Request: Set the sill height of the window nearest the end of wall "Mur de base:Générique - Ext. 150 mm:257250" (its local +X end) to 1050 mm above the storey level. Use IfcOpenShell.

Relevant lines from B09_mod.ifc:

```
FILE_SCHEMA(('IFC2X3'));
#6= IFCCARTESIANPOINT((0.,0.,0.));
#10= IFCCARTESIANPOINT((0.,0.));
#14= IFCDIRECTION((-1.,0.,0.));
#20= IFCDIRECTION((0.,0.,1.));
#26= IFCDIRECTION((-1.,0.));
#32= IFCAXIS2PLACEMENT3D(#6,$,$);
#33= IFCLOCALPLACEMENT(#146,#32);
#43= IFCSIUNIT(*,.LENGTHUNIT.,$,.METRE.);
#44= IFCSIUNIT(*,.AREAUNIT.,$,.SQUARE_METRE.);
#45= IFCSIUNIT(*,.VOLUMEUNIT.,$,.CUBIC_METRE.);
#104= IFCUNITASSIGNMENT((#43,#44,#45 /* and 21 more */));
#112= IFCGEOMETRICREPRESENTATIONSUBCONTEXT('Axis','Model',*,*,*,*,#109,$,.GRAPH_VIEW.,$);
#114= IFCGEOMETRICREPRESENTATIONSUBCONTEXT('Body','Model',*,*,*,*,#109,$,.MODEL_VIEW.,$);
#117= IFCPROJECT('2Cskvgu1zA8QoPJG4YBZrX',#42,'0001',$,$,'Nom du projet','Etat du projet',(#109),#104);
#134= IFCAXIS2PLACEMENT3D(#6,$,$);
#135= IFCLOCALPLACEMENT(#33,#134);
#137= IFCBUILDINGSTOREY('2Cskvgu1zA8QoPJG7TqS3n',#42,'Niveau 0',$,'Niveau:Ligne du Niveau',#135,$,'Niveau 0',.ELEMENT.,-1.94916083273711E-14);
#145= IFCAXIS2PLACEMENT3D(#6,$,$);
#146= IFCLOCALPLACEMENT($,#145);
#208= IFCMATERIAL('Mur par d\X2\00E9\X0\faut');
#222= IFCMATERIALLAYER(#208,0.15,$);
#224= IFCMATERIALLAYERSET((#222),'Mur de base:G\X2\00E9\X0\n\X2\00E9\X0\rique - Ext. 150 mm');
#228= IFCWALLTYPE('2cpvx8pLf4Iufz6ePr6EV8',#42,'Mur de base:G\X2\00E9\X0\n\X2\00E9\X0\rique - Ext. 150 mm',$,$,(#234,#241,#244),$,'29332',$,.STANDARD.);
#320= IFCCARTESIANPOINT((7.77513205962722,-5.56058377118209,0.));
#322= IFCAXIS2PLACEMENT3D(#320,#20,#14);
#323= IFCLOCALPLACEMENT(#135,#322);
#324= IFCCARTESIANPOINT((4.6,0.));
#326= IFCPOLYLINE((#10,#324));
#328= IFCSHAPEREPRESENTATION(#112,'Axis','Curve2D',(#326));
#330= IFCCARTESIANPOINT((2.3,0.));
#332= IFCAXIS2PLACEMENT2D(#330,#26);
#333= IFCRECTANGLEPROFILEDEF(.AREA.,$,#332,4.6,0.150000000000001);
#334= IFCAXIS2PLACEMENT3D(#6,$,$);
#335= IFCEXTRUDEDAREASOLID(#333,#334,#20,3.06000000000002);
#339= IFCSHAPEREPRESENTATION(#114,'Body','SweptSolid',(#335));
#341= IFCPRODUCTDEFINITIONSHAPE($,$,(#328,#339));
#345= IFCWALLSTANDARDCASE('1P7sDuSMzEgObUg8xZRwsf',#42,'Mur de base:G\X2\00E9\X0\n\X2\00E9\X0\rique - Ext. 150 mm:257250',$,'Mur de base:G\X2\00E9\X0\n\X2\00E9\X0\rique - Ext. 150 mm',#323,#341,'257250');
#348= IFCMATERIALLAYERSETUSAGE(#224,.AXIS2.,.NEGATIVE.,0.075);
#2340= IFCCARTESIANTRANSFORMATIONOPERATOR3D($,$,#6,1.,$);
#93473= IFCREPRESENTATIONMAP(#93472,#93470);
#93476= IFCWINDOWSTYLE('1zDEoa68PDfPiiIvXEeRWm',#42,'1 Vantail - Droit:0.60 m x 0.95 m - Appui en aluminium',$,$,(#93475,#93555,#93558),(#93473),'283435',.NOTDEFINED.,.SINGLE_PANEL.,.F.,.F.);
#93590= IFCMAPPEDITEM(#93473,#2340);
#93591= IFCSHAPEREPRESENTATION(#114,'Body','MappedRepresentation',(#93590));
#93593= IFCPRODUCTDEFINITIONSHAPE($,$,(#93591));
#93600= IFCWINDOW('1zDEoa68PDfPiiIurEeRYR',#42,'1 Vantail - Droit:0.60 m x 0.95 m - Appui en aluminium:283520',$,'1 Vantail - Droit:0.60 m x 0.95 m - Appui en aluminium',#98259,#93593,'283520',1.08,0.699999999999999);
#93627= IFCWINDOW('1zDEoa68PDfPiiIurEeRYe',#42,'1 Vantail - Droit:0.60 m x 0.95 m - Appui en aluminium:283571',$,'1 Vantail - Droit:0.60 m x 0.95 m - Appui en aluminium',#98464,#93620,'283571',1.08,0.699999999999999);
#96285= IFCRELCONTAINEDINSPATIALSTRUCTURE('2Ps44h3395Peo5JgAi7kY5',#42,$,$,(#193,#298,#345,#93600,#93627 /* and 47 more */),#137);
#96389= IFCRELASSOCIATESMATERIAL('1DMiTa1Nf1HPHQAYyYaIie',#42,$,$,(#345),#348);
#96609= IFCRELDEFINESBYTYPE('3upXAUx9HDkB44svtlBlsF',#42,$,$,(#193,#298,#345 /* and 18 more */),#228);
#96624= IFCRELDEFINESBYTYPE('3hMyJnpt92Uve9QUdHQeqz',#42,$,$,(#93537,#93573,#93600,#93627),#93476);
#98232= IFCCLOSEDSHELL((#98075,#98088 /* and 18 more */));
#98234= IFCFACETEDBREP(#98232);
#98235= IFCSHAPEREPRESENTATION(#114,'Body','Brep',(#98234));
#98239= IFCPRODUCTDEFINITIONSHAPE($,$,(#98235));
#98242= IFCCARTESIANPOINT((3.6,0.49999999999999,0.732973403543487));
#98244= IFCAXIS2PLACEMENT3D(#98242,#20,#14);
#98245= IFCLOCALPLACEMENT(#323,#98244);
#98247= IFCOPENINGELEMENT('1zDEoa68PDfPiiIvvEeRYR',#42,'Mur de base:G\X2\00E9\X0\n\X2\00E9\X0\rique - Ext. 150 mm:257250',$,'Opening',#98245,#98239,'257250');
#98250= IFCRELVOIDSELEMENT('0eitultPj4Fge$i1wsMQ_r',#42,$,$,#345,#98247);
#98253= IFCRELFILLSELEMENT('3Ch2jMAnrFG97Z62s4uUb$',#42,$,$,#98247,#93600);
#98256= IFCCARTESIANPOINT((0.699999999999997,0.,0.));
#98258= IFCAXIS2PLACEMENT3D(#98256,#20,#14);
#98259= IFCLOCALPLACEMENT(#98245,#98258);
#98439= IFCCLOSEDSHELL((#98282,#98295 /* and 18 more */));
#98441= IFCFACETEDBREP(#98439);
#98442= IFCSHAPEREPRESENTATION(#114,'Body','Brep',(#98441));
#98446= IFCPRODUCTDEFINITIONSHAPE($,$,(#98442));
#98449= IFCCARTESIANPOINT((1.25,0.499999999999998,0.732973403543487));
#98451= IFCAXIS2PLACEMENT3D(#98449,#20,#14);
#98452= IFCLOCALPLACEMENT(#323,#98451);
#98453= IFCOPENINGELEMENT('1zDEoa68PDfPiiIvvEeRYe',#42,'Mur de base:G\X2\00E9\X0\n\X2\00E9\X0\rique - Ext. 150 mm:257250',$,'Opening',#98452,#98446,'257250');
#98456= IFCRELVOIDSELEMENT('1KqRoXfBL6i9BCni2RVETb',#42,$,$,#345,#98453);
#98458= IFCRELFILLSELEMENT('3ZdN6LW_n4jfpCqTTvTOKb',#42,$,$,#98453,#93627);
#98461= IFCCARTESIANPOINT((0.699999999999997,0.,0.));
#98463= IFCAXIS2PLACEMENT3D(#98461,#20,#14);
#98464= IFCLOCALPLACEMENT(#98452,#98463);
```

```python
import numpy as np
import ifcopenshell
import ifcopenshell.api.geometry
import ifcopenshell.geom
import ifcopenshell.util.element
import ifcopenshell.util.placement
import ifcopenshell.util.shape
import ifcopenshell.util.unit

model = ifcopenshell.open("B09_mod.ifc")
unit_scale = ifcopenshell.util.unit.calculate_unit_scale(model)

window = model.by_id(93600)
opening = window.FillsVoids[0].RelatingOpeningElement
storey = ifcopenshell.util.element.get_container(window, ifc_class="IfcBuildingStorey")
level = ifcopenshell.util.placement.get_local_placement(storey.ObjectPlacement)[2, 3]

# The opening's origin need not be at the sill, so measure its lowest point.
shape = ifcopenshell.geom.create_shape(ifcopenshell.geom.settings(), opening)
bottom = ifcopenshell.util.shape.get_shape_bottom_elevation(shape, shape.geometry) / unit_scale
dz = level + 1.05 / unit_scale - bottom

shift = np.array([0.0, 0.0, dz])
# The window is placed relative to its opening, so it follows when the opening moves.
matrix = ifcopenshell.util.placement.get_local_placement(opening.ObjectPlacement)
matrix[:3, 3] += shift
ifcopenshell.api.geometry.edit_object_placement(
    model, product=opening, matrix=matrix, is_si=False, should_transform_children=True
)

print(f"moved by {dz * unit_scale:+.3f} m")

model.write("B09_mod_rev.ifc")
```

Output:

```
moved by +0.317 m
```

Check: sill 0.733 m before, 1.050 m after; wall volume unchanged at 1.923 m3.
